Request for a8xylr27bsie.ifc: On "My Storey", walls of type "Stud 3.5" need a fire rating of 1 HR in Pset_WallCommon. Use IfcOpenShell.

First a look at what the model holds.

```python
import ifcopenshell
import ifcopenshell.util.element

model = ifcopenshell.open("a8xylr27bsie.ifc")
print(model.schema)
storey = next(s for s in model.by_type("IfcBuildingStorey") if s.Name == "My Storey")
walls = [e for e in ifcopenshell.util.element.get_decomposition(storey) if e.is_a("IfcWall")]
seen = {}
for e in walls:
    element_type = ifcopenshell.util.element.get_type(e)
    key = (element_type.Name if element_type != e and element_type else None, ifcopenshell.util.element.get_pset(e, "Pset_WallCommon", "FireRating"))
    seen[key] = seen.get(key, 0) + 1
for (name, value), count in sorted(seen.items(), key=str):
    print(count, "x", name, "|", value)
```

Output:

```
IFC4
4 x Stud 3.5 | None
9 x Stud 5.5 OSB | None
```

```python
import ifcopenshell
import ifcopenshell.api.pset
import ifcopenshell.util.element

model = ifcopenshell.open("a8xylr27bsie.ifc")

storey = next(s for s in model.by_type("IfcBuildingStorey") if s.Name == "My Storey")
walls = [e for e in ifcopenshell.util.element.get_decomposition(storey) if e.is_a("IfcWall")]

count = 0
for e in walls:
    element_type = ifcopenshell.util.element.get_type(e)
    if element_type in (None, e) or element_type.Name != "Stud 3.5":
        continue
    # add_pset returns the element's existing set when there is one.
    pset = ifcopenshell.api.pset.add_pset(model, product=e, name="Pset_WallCommon")
    ifcopenshell.api.pset.edit_pset(model, pset=pset, properties={"FireRating": "1 HR"})
    count += 1

print(count, "walls updated")

model.write("a8xylr27bsie_updated.ifc")
```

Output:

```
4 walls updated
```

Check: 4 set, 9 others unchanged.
